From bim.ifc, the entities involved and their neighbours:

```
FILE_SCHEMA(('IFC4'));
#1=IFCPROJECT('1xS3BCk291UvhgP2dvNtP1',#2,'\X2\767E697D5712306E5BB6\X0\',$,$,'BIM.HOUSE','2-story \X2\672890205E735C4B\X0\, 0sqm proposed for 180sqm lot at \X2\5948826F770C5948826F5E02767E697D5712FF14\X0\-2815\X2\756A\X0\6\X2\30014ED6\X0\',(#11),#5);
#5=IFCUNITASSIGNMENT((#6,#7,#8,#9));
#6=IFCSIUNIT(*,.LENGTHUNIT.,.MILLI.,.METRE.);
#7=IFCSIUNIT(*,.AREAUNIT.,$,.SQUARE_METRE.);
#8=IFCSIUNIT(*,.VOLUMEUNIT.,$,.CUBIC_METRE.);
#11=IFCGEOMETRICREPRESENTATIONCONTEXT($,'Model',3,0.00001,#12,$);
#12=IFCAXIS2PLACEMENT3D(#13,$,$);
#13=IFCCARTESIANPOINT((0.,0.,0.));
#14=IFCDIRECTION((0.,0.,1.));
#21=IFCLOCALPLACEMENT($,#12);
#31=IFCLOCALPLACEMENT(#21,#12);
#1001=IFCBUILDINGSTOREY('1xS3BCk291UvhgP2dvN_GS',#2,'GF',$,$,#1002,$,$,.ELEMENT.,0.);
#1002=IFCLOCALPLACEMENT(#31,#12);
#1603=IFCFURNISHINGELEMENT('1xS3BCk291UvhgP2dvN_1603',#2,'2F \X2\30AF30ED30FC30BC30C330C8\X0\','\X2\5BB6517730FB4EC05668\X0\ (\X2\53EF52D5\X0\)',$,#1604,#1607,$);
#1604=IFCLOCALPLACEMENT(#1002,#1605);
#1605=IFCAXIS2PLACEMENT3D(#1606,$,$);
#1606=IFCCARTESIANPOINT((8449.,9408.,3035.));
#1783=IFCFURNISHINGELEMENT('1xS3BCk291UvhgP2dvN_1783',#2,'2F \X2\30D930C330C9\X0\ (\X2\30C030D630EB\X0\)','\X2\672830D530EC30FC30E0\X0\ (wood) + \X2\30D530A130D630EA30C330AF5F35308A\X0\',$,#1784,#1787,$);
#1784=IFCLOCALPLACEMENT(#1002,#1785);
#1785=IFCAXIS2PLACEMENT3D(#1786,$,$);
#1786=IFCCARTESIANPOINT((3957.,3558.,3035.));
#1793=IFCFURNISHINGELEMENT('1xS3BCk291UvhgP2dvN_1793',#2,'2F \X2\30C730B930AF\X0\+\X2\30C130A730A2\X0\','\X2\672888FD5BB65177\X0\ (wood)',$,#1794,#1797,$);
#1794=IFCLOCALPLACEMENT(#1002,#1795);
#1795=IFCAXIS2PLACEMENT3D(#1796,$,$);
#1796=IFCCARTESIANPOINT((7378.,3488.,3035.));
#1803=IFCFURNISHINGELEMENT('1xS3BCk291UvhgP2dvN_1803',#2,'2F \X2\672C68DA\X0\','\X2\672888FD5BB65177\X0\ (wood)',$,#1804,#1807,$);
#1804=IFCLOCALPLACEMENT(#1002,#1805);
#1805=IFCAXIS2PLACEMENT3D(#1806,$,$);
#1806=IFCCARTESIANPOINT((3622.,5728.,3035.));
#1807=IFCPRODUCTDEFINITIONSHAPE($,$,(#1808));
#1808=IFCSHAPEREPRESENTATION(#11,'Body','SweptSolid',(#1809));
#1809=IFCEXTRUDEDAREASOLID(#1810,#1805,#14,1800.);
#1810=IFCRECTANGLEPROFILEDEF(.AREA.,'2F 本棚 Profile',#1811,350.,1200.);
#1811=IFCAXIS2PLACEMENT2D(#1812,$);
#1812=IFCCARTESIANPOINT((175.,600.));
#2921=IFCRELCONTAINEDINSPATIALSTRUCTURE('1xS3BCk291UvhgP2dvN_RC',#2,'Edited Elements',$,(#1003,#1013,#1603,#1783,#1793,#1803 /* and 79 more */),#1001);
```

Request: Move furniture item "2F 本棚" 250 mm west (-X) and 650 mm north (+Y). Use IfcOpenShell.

```python
import ifcopenshell
import ifcopenshell.api.geometry
import ifcopenshell.util.placement
import ifcopenshell.util.unit

model = ifcopenshell.open("bim.ifc")
unit_scale = ifcopenshell.util.unit.calculate_unit_scale(model)

item = model.by_guid("1xS3BCk291UvhgP2dvN_1803")
matrix = ifcopenshell.util.placement.get_local_placement(item.ObjectPlacement)
matrix[0, 3] -= 0.25 / unit_scale
matrix[1, 3] += 0.65 / unit_scale
ifcopenshell.api.geometry.edit_object_placement(model, product=item, matrix=matrix, is_si=False)

print(ifcopenshell.util.placement.get_local_placement(item.ObjectPlacement).round(3) + 0.0)

model.write("bim_edited.ifc")
```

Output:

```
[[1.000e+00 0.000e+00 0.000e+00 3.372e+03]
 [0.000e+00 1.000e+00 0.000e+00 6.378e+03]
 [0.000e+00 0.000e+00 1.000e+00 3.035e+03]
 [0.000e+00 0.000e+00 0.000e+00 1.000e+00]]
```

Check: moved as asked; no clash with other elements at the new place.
